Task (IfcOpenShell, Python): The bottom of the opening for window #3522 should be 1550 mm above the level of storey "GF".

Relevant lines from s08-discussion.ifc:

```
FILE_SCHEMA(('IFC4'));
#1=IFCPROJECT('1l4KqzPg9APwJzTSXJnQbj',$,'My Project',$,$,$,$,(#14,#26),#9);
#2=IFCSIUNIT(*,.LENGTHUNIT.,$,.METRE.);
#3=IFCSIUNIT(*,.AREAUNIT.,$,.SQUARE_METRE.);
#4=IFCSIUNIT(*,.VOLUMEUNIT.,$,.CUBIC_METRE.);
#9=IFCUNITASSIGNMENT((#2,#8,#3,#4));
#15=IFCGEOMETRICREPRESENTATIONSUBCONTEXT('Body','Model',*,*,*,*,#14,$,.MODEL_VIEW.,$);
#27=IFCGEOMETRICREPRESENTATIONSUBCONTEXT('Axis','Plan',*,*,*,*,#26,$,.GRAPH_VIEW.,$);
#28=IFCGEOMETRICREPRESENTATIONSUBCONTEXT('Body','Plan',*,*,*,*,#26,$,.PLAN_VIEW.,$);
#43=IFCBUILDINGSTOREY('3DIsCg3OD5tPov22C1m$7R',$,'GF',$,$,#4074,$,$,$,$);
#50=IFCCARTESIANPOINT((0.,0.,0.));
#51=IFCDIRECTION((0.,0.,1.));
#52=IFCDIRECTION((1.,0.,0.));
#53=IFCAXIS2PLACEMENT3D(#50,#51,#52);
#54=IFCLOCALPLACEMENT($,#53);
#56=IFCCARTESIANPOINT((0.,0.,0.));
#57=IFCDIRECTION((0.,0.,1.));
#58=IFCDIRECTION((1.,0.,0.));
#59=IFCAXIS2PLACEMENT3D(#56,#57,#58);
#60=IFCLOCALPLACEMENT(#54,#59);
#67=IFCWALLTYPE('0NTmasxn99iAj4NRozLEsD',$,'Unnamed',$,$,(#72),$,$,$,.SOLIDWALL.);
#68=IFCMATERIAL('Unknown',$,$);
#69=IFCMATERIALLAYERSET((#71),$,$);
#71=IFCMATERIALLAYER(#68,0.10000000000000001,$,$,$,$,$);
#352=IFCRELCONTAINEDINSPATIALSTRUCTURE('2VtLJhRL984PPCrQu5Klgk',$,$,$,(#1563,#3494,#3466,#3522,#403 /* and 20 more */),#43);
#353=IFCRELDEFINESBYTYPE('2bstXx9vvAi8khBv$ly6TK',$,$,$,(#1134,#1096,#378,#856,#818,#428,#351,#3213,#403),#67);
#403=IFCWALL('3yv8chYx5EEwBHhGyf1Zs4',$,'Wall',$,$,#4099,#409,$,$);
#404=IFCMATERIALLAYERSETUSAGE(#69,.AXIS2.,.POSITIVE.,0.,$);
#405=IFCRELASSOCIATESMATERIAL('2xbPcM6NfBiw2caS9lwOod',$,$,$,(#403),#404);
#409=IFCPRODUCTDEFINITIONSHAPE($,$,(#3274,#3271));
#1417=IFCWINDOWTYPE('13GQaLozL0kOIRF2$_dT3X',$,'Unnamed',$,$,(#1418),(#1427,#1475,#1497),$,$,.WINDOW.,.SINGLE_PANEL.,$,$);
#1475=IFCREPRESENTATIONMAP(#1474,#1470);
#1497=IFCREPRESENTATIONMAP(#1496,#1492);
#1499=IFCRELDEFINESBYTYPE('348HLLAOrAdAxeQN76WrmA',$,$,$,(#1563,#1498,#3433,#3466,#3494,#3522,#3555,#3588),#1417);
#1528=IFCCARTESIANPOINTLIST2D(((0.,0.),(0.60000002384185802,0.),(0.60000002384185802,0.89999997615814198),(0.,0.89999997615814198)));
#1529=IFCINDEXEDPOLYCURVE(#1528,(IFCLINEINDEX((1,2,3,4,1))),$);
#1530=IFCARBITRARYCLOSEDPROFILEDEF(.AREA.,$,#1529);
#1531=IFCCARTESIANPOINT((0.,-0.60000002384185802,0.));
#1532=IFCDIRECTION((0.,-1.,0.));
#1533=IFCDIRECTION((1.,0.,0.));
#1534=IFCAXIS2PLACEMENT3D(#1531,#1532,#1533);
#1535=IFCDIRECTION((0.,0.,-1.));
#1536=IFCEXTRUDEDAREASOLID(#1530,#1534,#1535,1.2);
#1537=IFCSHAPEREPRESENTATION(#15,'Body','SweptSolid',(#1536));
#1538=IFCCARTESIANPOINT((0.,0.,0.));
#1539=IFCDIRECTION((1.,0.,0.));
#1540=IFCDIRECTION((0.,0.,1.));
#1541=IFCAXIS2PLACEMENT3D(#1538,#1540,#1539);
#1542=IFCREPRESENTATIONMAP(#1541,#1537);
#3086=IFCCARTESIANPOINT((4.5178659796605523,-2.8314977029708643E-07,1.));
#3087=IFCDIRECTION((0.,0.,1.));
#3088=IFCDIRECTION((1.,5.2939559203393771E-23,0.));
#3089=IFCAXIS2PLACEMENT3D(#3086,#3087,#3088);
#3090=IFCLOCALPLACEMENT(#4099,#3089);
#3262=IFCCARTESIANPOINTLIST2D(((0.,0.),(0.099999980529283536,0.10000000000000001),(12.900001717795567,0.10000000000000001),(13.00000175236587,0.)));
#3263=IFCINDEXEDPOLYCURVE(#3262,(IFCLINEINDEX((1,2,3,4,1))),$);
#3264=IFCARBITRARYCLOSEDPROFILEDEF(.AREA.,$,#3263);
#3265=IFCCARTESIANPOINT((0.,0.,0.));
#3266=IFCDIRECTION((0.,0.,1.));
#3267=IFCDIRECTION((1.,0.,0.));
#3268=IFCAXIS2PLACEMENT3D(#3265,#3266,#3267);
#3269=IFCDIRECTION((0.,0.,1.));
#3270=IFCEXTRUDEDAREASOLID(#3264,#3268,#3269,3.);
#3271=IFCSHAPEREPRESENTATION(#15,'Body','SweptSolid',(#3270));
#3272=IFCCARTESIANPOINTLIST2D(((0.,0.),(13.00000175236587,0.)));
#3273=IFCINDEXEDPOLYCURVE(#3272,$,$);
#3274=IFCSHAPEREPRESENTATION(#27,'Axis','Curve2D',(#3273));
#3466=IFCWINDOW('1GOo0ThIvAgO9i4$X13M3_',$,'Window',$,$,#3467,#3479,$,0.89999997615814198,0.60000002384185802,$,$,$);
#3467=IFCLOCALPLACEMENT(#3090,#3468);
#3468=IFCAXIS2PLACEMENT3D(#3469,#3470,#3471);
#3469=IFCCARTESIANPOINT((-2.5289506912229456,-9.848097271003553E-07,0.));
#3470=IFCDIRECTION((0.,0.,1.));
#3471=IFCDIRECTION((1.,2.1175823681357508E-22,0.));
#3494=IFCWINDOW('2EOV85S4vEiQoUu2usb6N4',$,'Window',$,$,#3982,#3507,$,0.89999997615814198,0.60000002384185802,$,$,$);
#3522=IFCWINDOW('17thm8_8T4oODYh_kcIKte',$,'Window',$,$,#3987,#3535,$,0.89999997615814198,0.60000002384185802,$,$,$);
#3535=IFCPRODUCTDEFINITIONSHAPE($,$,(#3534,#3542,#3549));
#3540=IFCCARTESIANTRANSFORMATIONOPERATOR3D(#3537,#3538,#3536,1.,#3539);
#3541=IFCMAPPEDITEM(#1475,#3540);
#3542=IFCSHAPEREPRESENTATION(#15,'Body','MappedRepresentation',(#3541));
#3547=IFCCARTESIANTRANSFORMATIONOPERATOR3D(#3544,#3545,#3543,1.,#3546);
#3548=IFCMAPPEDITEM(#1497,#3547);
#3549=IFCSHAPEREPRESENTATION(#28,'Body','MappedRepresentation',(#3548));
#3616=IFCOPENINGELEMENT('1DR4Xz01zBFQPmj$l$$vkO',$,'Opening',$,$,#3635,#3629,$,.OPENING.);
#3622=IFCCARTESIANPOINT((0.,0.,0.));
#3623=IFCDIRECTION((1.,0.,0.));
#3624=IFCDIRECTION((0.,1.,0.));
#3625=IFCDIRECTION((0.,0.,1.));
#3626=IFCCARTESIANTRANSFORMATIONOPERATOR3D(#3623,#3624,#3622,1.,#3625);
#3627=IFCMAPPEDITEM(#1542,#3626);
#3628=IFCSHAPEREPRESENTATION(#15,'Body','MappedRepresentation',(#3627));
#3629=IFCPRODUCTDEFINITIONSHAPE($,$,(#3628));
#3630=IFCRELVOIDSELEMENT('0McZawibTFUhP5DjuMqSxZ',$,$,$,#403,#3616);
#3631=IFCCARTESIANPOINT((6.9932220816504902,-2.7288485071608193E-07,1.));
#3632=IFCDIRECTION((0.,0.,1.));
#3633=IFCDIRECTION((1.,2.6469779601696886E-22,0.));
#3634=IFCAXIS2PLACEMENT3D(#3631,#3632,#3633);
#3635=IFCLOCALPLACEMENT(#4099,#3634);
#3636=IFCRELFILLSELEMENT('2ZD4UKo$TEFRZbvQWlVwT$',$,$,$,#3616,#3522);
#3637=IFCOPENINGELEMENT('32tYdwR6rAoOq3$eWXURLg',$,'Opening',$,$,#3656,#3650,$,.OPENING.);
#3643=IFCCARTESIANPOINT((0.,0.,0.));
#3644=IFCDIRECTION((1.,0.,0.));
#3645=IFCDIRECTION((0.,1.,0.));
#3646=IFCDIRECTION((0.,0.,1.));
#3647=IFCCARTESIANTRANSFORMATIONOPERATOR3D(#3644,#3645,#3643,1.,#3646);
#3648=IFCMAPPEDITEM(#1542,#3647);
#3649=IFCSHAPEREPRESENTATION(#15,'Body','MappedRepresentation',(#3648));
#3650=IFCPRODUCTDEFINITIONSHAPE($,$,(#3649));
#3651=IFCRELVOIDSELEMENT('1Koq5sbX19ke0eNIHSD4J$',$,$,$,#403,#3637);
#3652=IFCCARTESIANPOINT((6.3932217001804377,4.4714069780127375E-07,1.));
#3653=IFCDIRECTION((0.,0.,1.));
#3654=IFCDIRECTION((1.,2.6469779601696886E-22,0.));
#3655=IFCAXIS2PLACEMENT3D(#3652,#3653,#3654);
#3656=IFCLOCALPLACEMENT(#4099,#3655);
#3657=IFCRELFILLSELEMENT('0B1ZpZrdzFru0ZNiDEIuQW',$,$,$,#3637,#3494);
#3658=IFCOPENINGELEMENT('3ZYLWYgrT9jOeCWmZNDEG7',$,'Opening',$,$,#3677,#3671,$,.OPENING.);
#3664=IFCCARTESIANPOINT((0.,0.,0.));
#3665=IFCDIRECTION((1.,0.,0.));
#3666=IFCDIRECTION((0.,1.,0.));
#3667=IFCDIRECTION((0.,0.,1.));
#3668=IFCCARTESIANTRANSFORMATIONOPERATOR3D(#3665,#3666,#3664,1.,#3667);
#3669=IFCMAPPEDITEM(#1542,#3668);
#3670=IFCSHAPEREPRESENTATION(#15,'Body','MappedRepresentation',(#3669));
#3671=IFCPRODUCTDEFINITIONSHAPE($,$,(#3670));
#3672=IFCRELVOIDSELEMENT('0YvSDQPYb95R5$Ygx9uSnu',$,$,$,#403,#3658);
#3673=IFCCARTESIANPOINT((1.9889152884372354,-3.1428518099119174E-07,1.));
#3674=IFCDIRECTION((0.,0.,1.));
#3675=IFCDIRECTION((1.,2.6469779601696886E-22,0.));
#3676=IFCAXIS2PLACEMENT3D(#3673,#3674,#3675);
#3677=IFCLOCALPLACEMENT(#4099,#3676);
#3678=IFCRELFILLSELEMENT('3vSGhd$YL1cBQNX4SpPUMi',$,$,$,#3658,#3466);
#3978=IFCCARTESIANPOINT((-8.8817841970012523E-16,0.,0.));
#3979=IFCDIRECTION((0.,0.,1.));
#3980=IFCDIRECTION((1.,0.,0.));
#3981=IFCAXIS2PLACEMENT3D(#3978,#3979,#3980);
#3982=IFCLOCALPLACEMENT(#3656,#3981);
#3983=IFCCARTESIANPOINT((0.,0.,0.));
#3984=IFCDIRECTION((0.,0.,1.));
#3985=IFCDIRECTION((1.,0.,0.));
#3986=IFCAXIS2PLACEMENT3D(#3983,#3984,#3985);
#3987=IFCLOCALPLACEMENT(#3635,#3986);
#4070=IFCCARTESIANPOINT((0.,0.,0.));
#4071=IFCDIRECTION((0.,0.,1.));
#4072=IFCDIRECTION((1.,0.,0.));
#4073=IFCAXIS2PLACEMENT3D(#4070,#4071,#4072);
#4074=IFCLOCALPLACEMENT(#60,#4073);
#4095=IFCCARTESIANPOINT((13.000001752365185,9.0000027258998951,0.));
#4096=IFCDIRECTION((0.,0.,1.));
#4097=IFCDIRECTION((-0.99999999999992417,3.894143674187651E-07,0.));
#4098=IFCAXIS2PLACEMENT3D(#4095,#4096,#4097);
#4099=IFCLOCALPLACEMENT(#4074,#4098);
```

```python
import numpy as np
import ifcopenshell
import ifcopenshell.api.geometry
import ifcopenshell.geom
import ifcopenshell.util.element
import ifcopenshell.util.placement
import ifcopenshell.util.shape
import ifcopenshell.util.unit

model = ifcopenshell.open("s08-discussion.ifc")
unit_scale = ifcopenshell.util.unit.calculate_unit_scale(model)

window = model.by_guid("17thm8_8T4oODYh_kcIKte")
opening = window.FillsVoids[0].RelatingOpeningElement
storey = ifcopenshell.util.element.get_container(window, ifc_class="IfcBuildingStorey")
level = ifcopenshell.util.placement.get_local_placement(storey.ObjectPlacement)[2, 3]

# The opening's origin need not be at the sill, so measure its lowest point.
shape = ifcopenshell.geom.create_shape(ifcopenshell.geom.settings(), opening)
bottom = ifcopenshell.util.shape.get_shape_bottom_elevation(shape, shape.geometry) / unit_scale
dz = level + 1.55 / unit_scale - bottom

shift = np.array([0.0, 0.0, dz])
# The window is placed relative to its opening, so it follows when the opening moves.
matrix = ifcopenshell.util.placement.get_local_placement(opening.ObjectPlacement)
matrix[:3, 3] += shift
ifcopenshell.api.geometry.edit_object_placement(
    model, product=opening, matrix=matrix, is_si=False, should_transform_children=True
)

print(f"moved by {dz * unit_scale:+.3f} m")

model.write("s08-discussion_updated.ifc")
```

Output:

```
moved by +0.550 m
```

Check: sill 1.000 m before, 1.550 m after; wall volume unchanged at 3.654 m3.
